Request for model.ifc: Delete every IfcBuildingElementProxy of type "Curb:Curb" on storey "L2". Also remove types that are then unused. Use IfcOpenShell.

First a look at what the model holds.

```python
import ifcopenshell
import ifcopenshell.util.element

model = ifcopenshell.open("model.ifc")
print(model.schema)
storey = next(s for s in model.by_type("IfcBuildingStorey") if s.Name == "L2")
proxies = [e for e in ifcopenshell.util.element.get_decomposition(storey) if e.is_a("IfcBuildingElementProxy")]
seen = {}
for e in proxies:
    element_type = ifcopenshell.util.element.get_type(e)
    name = element_type.Name if element_type not in (None, e) else None
    seen[name] = seen.get(name, 0) + 1
for name, count in sorted(seen.items(), key=str):
    print(count, "x", name)
```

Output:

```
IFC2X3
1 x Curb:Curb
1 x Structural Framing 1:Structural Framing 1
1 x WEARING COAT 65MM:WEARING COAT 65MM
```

```python
import ifcopenshell
import ifcopenshell.api.root
import ifcopenshell.util.element

model = ifcopenshell.open("model.ifc")

storey = next(s for s in model.by_type("IfcBuildingStorey") if s.Name == "L2")
proxies = [e for e in ifcopenshell.util.element.get_decomposition(storey) if e.is_a("IfcBuildingElementProxy")]
targets = [e for e in proxies if (t := ifcopenshell.util.element.get_type(e)) not in (None, e) and t.Name == "Curb:Curb"]
types = {ifcopenshell.util.element.get_type(e) for e in targets} - {None, *targets}

for e in targets:
    ifcopenshell.api.root.remove_product(model, product=e)
print(len(targets), "removed")

unused = [t for t in types if not ifcopenshell.util.element.get_types(t)]
for t in unused:
    ifcopenshell.api.root.remove_product(model, product=t)
print(len(unused), "unused types removed")

model.write("model_v2.ifc")
```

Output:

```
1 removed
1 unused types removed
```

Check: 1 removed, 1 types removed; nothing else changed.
